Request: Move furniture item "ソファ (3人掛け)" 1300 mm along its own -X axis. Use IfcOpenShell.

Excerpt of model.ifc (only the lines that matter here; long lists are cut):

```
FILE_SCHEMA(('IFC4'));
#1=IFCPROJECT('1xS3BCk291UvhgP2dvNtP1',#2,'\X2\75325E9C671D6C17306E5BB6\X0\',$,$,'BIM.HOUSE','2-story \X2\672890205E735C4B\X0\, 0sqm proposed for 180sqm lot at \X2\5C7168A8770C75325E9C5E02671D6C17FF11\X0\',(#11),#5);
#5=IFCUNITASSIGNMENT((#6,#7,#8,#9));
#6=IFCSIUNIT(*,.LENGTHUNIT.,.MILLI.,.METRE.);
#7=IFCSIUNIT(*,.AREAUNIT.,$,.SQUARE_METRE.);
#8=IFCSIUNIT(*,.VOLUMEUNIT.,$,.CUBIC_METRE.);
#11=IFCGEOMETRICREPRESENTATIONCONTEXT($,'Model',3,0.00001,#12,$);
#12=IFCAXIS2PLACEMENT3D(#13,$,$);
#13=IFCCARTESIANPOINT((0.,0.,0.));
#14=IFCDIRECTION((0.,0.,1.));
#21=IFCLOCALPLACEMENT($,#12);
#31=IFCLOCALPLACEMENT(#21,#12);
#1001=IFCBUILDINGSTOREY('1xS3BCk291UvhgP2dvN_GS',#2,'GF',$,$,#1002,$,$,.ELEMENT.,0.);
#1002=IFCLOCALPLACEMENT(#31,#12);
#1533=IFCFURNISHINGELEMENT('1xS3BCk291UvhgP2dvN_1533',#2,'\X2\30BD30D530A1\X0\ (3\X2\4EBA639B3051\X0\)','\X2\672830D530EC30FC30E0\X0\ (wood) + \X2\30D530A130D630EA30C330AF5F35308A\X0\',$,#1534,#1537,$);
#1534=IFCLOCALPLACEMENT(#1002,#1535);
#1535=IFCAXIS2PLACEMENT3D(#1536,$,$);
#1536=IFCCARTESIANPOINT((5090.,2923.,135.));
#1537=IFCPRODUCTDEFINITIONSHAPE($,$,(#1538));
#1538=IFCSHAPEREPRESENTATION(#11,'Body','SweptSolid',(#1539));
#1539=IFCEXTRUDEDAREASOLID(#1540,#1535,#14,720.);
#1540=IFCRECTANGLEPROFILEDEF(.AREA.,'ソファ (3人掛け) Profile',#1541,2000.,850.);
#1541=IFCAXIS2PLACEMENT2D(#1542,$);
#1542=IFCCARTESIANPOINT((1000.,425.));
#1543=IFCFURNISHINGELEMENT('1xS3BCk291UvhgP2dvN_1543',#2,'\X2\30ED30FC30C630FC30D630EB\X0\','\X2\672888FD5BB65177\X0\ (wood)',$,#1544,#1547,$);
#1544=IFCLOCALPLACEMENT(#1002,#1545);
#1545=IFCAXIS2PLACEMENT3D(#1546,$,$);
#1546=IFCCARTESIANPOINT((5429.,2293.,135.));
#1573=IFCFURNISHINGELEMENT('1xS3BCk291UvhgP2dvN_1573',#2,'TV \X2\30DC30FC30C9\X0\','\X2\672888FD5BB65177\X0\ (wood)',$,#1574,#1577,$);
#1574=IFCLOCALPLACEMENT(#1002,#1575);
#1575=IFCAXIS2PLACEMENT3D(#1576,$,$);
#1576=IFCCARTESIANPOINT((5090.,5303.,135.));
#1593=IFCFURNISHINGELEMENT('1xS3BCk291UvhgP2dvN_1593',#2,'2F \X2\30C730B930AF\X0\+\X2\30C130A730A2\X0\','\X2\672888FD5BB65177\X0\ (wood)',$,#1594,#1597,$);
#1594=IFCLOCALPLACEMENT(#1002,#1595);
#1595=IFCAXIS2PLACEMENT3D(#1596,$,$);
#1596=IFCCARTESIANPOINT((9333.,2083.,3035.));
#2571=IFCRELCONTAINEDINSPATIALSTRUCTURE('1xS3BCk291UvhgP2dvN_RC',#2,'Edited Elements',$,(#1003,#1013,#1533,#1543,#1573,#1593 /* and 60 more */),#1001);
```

```python
import ifcopenshell
import ifcopenshell.api.geometry
import ifcopenshell.util.placement

model = ifcopenshell.open("model.ifc")

item = model.by_id(1533)
matrix = ifcopenshell.util.placement.get_local_placement(item.ObjectPlacement)
matrix[:3, 3] -= matrix[:3, 0] * 1300.0
ifcopenshell.api.geometry.edit_object_placement(model, product=item, matrix=matrix, is_si=False)

print(ifcopenshell.util.placement.get_local_placement(item.ObjectPlacement).round(3) + 0.0)

model.write("model-out.ifc")
```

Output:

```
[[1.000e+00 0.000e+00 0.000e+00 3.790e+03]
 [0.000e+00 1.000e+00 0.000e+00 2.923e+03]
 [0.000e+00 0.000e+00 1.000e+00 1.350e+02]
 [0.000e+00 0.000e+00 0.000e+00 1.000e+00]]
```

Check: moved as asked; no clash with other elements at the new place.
